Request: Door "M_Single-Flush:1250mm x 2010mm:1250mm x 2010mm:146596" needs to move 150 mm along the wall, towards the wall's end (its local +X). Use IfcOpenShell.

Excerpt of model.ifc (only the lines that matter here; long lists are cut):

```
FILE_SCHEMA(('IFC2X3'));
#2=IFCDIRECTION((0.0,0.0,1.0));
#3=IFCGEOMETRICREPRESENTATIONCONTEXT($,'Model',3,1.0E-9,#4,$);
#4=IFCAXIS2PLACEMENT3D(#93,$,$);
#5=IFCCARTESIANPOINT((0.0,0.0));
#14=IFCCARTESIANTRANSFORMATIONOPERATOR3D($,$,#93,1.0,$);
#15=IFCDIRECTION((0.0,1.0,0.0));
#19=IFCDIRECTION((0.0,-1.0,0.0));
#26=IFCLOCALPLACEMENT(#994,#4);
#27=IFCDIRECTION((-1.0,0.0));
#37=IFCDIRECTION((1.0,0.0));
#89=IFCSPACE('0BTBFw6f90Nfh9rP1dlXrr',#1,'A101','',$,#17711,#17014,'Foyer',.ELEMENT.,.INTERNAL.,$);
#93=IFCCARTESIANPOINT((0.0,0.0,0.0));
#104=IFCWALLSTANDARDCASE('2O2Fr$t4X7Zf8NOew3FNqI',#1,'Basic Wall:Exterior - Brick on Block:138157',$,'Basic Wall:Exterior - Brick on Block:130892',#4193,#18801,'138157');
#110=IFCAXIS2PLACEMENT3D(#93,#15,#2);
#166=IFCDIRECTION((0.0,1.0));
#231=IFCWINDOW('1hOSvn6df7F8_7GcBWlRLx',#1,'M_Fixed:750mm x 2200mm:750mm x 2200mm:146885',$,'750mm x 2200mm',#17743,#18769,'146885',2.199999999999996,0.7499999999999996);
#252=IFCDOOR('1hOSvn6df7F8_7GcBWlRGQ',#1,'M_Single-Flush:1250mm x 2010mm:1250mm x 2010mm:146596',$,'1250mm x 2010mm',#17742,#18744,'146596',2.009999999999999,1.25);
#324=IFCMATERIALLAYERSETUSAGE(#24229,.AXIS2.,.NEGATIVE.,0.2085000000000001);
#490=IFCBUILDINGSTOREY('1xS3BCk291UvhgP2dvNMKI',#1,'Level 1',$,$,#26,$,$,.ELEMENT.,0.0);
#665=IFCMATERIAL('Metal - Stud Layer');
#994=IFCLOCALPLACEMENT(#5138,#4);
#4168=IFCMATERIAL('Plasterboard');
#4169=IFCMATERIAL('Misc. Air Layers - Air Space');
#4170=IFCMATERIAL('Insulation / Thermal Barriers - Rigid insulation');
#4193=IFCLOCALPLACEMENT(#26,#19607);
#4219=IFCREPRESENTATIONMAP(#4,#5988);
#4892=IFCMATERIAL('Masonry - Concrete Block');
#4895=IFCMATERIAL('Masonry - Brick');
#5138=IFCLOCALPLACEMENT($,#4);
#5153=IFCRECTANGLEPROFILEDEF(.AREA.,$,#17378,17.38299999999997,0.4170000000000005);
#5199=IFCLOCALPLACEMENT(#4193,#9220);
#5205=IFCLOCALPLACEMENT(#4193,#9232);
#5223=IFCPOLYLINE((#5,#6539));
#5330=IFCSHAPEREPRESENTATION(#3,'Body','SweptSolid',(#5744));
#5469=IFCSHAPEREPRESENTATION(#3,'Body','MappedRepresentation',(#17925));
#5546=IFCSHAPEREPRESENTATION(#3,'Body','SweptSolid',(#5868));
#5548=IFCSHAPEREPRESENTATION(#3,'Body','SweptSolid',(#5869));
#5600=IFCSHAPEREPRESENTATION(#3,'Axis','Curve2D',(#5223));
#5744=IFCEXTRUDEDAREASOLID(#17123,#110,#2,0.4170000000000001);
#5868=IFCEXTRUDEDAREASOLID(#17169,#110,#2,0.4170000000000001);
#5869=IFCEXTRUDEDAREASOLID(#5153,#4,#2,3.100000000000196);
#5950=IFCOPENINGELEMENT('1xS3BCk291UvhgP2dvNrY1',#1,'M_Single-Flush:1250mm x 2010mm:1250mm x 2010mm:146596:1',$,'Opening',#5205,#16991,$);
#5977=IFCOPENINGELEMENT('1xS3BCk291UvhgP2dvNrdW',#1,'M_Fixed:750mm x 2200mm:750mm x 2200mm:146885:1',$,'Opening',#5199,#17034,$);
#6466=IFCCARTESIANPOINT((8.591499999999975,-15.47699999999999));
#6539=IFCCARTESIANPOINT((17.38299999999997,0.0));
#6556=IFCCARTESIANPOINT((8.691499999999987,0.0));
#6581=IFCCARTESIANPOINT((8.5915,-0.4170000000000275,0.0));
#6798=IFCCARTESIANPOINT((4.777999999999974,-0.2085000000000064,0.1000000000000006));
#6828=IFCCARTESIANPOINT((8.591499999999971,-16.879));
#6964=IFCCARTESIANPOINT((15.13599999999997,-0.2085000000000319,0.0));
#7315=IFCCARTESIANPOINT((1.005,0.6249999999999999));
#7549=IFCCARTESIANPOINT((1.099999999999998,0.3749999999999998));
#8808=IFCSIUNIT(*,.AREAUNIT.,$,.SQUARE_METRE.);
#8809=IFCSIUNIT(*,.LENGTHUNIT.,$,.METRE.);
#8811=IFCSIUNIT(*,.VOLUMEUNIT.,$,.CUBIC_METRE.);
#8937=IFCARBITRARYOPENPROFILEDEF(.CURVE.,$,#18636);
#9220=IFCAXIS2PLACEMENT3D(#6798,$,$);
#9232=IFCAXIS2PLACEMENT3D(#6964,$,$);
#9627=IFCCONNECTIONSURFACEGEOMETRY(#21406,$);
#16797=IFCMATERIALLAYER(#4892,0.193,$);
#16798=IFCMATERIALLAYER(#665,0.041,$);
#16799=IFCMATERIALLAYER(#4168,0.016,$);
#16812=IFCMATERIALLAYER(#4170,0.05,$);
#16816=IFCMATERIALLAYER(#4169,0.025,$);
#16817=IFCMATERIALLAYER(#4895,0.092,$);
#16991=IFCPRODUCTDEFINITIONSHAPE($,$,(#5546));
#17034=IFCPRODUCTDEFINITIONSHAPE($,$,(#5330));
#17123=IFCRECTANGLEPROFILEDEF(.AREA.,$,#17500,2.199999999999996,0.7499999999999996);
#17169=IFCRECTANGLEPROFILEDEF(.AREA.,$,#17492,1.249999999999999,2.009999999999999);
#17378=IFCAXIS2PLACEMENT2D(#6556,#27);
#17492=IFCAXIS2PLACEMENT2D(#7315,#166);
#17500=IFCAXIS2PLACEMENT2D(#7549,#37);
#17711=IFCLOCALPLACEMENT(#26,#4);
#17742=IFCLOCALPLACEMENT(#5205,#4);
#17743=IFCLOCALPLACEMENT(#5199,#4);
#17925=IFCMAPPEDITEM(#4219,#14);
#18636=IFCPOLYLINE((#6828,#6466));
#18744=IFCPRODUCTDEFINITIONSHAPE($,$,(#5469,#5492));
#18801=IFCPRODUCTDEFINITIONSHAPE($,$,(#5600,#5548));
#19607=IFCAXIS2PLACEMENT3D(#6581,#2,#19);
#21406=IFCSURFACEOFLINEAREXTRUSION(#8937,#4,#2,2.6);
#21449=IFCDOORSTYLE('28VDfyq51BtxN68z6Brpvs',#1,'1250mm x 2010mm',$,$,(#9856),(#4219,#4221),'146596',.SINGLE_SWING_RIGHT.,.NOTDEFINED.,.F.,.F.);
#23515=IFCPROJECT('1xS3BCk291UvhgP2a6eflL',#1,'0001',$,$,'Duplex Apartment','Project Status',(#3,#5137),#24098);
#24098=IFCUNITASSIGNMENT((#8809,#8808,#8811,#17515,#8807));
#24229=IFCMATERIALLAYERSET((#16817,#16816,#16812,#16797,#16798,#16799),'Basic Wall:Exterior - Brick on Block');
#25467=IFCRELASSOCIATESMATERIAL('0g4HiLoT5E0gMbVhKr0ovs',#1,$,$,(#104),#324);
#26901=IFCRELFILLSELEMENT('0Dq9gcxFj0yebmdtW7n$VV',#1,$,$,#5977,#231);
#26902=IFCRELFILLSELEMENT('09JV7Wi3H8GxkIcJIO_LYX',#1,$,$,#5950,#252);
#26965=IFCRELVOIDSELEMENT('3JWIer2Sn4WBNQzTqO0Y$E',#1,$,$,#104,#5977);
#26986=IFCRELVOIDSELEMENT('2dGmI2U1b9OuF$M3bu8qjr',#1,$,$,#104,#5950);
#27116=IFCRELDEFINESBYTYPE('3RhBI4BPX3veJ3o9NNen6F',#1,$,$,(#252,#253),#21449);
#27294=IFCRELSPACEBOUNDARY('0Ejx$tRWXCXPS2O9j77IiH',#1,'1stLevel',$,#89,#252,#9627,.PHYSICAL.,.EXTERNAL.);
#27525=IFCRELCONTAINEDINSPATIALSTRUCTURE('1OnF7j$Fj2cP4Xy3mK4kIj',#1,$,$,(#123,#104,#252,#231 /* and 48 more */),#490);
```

```python
import numpy as np
import ifcopenshell
import ifcopenshell.api.geometry
import ifcopenshell.util.placement
import ifcopenshell.util.unit

model = ifcopenshell.open("model.ifc")
unit_scale = ifcopenshell.util.unit.calculate_unit_scale(model)

door = model.by_id(252)
opening = door.FillsVoids[0].RelatingOpeningElement
wall = opening.VoidsElements[0].RelatingBuildingElement

wall_matrix = ifcopenshell.util.placement.get_local_placement(wall.ObjectPlacement)
shift = wall_matrix[:3, 0] * 0.15 / unit_scale
before = ifcopenshell.util.placement.get_local_placement(door.ObjectPlacement)[:3, 3].copy()

# The door is placed relative to its opening, so it follows when the opening moves.
matrix = ifcopenshell.util.placement.get_local_placement(opening.ObjectPlacement)
matrix[:3, 3] += shift
ifcopenshell.api.geometry.edit_object_placement(
    model, product=opening, matrix=matrix, is_si=False, should_transform_children=True
)

# Space boundary surfaces are stored in each space's coordinates; move them too.
for rel in door.ProvidesBoundaries:
    if not rel.ConnectionGeometry:
        continue
    surface = rel.ConnectionGeometry.SurfaceOnRelatingElement
    space_matrix = ifcopenshell.util.placement.get_local_placement(rel.RelatingSpace.ObjectPlacement)
    point = np.array(surface.Position.Location.Coordinates) + space_matrix[:3, :3].T @ shift
    surface.Position = model.createIfcAxis2Placement3D(
        model.createIfcCartesianPoint(point.tolist()), surface.Position.Axis, surface.Position.RefDirection
    )

after = ifcopenshell.util.placement.get_local_placement(door.ObjectPlacement)[:3, 3]
print("door moved by", (after - before).round(3) + 0.0)

model.write("model_v2.ifc")
```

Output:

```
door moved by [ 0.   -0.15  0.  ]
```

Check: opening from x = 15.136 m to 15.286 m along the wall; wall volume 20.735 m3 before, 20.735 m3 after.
